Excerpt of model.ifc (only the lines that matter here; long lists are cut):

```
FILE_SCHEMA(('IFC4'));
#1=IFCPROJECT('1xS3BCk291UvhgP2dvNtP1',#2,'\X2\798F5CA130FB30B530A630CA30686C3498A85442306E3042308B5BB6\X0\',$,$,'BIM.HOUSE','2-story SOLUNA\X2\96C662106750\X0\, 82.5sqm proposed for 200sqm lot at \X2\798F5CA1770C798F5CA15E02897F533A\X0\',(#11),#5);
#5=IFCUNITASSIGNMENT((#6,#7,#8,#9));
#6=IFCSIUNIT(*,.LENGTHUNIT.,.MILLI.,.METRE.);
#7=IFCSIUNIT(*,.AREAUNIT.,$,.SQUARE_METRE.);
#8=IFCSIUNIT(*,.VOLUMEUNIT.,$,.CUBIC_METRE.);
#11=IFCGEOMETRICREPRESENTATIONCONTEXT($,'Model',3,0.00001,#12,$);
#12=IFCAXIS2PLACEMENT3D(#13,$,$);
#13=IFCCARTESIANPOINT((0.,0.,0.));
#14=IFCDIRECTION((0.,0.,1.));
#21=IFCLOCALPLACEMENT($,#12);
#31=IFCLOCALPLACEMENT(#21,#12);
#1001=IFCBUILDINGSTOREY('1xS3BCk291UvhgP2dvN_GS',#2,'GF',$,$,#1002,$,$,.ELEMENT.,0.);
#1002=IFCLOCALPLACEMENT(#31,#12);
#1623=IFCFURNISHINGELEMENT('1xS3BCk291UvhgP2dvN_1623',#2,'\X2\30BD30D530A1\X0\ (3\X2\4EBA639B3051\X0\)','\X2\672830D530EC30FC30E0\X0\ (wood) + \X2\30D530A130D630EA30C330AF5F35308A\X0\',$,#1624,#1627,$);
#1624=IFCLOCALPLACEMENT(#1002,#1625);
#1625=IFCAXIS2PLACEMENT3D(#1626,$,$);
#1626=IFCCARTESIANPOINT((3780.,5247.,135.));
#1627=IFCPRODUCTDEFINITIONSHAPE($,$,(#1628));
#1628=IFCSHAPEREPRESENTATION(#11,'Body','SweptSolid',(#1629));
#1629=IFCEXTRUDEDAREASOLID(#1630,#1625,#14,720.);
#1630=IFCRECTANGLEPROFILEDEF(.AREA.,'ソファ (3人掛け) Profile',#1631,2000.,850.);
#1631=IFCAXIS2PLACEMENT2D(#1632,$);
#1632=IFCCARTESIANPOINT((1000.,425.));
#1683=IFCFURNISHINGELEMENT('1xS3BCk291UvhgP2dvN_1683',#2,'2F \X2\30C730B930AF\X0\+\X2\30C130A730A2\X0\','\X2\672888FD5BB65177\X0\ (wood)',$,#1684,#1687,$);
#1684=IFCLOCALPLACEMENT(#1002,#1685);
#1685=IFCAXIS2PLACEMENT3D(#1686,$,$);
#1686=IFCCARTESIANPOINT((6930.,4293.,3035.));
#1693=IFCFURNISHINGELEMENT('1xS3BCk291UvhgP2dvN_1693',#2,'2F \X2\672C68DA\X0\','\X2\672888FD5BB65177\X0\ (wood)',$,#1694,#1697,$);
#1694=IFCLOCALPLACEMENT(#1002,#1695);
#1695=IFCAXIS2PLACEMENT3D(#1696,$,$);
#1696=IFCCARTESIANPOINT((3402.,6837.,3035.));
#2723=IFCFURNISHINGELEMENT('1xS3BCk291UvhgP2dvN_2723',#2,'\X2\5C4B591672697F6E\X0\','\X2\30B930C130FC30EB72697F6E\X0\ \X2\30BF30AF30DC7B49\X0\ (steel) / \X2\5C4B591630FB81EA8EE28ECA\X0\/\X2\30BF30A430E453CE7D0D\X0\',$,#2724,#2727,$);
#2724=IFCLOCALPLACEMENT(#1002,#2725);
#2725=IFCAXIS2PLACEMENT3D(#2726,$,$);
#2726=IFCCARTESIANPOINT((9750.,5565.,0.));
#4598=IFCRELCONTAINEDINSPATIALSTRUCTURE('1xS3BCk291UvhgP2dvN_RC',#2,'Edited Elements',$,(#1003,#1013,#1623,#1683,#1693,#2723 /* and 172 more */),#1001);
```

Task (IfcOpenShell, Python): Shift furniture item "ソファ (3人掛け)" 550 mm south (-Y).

```python
import ifcopenshell
import ifcopenshell.api.geometry
import ifcopenshell.util.placement

model = ifcopenshell.open("model.ifc")

item = model.by_id(1623)
matrix = ifcopenshell.util.placement.get_local_placement(item.ObjectPlacement)
matrix[1, 3] -= 550.0
ifcopenshell.api.geometry.edit_object_placement(model, product=item, matrix=matrix, is_si=False)

print(ifcopenshell.util.placement.get_local_placement(item.ObjectPlacement).round(3) + 0.0)

model.write("model_rev.ifc")
```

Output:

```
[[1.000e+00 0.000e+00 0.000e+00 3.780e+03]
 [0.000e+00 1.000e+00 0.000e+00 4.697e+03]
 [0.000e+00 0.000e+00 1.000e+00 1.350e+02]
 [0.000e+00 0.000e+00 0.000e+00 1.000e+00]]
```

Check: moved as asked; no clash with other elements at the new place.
